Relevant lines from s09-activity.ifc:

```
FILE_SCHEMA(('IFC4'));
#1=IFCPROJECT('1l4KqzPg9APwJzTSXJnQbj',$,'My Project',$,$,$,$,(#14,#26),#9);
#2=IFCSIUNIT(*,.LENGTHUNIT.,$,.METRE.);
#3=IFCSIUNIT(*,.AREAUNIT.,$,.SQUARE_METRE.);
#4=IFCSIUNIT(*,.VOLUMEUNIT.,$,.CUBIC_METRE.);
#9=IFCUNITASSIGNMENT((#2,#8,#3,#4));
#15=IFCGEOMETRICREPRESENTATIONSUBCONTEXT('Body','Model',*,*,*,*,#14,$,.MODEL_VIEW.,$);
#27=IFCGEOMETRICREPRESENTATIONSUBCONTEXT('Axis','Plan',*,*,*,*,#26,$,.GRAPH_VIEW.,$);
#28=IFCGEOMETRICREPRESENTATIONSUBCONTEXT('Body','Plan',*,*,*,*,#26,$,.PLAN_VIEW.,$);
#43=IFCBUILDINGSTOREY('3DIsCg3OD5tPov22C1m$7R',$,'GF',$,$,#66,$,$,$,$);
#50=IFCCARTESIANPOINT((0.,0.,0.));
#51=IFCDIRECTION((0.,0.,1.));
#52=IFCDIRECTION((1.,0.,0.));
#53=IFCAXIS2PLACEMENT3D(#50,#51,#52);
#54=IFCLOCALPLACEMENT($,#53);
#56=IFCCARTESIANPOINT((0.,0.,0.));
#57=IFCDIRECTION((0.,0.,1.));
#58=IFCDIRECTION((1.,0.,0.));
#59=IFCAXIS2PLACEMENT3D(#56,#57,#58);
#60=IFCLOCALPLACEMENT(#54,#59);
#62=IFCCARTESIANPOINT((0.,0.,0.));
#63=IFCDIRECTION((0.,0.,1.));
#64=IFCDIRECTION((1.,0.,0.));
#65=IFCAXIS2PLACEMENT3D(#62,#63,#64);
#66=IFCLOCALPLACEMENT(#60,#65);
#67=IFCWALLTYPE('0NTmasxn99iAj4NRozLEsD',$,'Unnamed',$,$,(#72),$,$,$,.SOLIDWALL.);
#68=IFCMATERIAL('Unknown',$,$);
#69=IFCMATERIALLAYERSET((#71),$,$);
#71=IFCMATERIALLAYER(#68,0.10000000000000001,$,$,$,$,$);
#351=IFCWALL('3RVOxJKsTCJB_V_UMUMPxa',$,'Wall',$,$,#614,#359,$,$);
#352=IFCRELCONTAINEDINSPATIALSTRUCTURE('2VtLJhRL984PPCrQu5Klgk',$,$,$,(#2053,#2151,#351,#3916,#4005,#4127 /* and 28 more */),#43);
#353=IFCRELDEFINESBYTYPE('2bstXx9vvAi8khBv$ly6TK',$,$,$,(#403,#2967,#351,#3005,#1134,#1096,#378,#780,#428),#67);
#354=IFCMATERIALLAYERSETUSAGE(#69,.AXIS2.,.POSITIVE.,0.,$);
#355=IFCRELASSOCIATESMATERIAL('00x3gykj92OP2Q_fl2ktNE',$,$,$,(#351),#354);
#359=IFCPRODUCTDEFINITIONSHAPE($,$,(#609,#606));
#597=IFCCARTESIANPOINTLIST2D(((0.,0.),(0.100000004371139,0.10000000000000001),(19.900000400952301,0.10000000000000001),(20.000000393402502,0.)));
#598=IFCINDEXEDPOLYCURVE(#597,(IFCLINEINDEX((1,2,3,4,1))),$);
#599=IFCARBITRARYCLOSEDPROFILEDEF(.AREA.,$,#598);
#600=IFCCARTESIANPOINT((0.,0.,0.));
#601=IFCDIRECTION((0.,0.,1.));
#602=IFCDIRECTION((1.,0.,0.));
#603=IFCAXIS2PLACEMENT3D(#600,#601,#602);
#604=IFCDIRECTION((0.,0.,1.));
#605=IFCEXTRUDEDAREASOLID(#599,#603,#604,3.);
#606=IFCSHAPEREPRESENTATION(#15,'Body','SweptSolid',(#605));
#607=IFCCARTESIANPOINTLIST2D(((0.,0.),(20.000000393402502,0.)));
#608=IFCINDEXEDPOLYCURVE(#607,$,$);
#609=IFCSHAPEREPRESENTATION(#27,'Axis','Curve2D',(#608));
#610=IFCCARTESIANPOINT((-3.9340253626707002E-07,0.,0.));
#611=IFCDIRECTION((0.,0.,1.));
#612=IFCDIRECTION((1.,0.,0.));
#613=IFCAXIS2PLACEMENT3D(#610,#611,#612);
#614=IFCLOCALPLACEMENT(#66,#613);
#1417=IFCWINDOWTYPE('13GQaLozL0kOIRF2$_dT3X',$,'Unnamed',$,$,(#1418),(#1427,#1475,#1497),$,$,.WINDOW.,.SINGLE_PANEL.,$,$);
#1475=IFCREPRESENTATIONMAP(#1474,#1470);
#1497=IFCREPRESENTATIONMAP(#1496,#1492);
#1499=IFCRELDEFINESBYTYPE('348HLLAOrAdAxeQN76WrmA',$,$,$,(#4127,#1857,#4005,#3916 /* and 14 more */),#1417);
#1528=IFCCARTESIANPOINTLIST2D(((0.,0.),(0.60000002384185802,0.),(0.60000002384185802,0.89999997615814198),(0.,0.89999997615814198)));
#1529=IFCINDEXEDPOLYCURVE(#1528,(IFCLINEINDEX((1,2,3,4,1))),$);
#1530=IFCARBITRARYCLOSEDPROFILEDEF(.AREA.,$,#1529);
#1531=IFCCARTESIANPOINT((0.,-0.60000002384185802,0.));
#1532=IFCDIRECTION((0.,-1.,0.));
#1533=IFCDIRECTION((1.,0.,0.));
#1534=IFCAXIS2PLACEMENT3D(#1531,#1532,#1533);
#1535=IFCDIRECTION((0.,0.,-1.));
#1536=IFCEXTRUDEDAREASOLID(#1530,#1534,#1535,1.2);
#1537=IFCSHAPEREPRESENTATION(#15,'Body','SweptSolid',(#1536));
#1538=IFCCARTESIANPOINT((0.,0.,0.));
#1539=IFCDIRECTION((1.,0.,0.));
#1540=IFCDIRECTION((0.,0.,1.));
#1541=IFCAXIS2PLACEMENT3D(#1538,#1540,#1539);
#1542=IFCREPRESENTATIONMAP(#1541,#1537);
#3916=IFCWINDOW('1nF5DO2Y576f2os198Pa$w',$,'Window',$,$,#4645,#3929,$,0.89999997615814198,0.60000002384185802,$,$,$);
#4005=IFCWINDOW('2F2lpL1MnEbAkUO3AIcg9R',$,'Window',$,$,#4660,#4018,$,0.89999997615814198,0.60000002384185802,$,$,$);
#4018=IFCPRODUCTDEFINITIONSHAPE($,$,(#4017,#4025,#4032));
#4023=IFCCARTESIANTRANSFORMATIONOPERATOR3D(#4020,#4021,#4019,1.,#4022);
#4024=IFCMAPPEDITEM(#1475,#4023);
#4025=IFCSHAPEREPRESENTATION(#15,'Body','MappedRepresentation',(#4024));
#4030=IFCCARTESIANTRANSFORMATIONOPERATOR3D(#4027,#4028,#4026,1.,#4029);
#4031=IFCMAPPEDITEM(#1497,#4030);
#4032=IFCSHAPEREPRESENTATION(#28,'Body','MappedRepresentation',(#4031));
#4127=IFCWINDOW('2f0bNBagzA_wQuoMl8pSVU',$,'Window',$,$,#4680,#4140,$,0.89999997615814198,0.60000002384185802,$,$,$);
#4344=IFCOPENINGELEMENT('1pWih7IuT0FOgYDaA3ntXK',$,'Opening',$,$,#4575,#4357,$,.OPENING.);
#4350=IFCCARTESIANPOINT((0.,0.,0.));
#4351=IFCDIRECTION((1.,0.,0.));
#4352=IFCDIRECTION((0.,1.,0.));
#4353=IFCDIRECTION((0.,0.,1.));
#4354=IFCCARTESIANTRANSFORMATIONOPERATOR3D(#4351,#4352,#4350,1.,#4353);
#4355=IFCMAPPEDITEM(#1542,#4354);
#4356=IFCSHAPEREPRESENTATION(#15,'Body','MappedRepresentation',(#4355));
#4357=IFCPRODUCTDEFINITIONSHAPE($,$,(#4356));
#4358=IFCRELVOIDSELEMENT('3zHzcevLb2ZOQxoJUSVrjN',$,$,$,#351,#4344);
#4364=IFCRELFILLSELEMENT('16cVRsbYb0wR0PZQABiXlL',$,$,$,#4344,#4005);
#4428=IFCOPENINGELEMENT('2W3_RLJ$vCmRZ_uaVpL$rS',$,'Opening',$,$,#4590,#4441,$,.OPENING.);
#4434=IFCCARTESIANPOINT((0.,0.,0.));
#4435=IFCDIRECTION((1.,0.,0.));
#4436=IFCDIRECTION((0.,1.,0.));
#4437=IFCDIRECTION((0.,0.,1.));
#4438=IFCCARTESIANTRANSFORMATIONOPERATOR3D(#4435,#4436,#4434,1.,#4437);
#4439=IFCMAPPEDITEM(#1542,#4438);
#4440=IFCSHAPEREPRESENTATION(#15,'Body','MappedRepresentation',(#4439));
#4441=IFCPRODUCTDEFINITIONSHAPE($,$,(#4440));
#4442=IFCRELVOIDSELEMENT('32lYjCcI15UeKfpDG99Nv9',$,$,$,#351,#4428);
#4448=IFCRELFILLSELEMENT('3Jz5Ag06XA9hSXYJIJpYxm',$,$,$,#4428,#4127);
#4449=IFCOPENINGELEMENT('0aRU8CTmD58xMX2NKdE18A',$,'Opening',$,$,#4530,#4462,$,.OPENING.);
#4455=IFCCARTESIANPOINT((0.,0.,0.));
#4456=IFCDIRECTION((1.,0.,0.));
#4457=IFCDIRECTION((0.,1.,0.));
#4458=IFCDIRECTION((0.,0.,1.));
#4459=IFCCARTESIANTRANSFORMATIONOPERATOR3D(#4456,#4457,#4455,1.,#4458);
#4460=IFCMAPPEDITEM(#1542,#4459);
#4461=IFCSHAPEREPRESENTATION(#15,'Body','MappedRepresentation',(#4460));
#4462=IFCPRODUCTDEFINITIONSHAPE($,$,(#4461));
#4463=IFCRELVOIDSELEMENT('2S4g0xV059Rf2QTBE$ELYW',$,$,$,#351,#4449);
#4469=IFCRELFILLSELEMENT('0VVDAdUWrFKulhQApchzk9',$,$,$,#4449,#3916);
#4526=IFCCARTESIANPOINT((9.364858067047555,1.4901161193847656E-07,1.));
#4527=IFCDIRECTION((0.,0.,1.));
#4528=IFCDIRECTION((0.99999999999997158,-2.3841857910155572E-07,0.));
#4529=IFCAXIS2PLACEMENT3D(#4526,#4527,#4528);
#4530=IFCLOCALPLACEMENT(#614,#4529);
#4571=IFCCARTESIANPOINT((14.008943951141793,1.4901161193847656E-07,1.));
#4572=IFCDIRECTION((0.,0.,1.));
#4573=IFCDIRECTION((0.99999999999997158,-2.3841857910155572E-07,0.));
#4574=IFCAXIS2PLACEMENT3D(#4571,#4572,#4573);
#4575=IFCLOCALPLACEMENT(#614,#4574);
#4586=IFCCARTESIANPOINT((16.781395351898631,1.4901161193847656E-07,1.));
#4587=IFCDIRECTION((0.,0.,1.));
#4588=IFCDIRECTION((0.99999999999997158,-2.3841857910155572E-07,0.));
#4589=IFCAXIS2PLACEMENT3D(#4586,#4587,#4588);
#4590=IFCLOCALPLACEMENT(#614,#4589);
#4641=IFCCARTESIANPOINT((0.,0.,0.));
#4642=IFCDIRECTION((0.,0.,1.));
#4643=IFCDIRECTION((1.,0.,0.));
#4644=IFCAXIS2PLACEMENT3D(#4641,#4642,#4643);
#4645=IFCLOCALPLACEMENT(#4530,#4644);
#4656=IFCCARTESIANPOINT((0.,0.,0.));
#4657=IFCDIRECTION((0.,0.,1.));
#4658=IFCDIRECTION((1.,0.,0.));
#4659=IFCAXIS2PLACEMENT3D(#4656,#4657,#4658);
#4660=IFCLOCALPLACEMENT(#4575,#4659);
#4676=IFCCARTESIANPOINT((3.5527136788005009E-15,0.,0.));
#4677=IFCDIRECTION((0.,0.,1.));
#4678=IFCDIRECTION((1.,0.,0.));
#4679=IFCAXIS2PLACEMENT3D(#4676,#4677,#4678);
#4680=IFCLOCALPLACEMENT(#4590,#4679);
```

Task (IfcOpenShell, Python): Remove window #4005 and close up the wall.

```python
import ifcopenshell
import ifcopenshell.api.feature
import ifcopenshell.api.root
import ifcopenshell.geom
import ifcopenshell.util.shape

model = ifcopenshell.open("s09-activity.ifc")
settings = ifcopenshell.geom.settings()


def volume(element):
    """Net volume in cubic metres, openings subtracted."""
    shape = ifcopenshell.geom.create_shape(settings, element)
    return ifcopenshell.util.shape.get_volume(shape.geometry)


window = model.by_id(4005)
opening = window.FillsVoids[0].RelatingOpeningElement
wall = opening.VoidsElements[0].RelatingBuildingElement
before = volume(wall)

ifcopenshell.api.root.remove_product(model, product=window)
ifcopenshell.api.feature.remove_feature(model, feature=opening)

after = volume(wall)

print(f"wall volume {before:.3f} -> {after:.3f} m3")

model.write("s09-activity_edited.ifc")
```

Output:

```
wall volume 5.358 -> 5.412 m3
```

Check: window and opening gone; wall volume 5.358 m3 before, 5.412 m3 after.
